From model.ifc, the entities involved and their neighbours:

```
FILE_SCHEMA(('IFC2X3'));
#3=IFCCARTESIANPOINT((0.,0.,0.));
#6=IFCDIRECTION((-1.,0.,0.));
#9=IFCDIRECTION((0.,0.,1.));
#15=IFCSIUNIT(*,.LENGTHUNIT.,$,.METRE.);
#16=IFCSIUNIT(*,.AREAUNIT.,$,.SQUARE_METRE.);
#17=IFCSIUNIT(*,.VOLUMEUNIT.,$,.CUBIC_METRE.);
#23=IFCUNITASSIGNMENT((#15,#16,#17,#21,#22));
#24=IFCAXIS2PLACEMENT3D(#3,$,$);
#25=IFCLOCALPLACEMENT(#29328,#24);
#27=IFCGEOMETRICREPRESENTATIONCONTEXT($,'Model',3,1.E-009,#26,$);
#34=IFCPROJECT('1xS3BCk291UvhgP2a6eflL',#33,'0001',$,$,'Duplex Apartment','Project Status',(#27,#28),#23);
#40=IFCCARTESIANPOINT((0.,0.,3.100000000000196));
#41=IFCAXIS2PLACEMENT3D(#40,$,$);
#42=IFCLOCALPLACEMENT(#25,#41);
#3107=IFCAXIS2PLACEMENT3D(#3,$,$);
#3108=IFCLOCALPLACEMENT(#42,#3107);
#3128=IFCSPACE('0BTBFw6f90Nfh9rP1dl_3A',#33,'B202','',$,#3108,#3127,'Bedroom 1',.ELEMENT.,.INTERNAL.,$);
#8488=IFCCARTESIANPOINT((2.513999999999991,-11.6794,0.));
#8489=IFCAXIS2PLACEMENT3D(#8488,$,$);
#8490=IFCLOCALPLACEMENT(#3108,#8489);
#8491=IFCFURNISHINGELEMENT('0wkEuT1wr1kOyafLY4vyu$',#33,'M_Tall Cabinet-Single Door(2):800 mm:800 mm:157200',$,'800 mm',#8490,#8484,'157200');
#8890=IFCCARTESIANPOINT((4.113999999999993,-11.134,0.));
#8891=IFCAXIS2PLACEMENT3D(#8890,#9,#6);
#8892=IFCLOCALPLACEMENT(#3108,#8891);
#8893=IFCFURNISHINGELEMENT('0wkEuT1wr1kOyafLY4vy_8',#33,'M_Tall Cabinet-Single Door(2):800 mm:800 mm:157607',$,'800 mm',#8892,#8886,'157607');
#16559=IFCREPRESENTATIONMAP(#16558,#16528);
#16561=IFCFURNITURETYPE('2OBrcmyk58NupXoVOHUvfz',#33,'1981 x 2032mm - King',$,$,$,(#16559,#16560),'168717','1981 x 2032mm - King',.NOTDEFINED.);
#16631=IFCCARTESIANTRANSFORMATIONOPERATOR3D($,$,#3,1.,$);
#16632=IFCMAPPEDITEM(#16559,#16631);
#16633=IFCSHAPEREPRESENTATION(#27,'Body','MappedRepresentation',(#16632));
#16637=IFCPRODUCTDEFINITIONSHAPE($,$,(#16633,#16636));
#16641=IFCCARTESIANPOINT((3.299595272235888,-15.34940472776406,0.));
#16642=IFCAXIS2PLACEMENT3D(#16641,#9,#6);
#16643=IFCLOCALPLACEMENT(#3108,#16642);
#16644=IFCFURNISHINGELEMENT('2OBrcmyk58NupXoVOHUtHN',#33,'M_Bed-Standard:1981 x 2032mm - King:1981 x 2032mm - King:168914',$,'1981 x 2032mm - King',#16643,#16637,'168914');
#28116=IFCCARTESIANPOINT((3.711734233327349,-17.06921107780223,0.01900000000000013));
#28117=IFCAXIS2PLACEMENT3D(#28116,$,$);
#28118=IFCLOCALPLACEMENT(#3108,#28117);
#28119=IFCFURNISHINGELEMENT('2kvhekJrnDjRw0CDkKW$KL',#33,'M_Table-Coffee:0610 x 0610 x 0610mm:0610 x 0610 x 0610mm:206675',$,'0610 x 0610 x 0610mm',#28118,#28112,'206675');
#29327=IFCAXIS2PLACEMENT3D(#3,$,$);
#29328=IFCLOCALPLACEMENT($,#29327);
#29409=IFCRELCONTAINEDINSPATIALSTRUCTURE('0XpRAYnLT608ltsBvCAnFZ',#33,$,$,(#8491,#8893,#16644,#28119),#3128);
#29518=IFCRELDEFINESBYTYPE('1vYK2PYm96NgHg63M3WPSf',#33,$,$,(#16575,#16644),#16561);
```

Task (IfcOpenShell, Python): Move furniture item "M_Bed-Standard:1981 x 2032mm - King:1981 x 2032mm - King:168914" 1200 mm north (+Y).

```python
import ifcopenshell
import ifcopenshell.api.geometry
import ifcopenshell.util.placement
import ifcopenshell.util.unit

model = ifcopenshell.open("model.ifc")
unit_scale = ifcopenshell.util.unit.calculate_unit_scale(model)

item = model.by_guid("2OBrcmyk58NupXoVOHUtHN")
matrix = ifcopenshell.util.placement.get_local_placement(item.ObjectPlacement)
matrix[1, 3] += 1.2 / unit_scale
ifcopenshell.api.geometry.edit_object_placement(model, product=item, matrix=matrix, is_si=False)

print(ifcopenshell.util.placement.get_local_placement(item.ObjectPlacement).round(3) + 0.0)

model.write("model-out.ifc")
```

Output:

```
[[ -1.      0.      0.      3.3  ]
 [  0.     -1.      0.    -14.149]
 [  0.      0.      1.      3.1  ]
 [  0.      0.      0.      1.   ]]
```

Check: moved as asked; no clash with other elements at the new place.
